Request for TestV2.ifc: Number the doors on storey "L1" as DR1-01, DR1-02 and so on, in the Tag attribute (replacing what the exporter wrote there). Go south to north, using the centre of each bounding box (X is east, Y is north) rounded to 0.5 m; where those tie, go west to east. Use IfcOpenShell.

First a look at what the model holds.

```python
import ifcopenshell
import ifcopenshell.util.element
import ifcopenshell.util.placement

model = ifcopenshell.open("TestV2.ifc")
print(model.schema)
storey = next(s for s in model.by_type("IfcBuildingStorey") if s.Name == "L1")
doors = [e for e in ifcopenshell.util.element.get_decomposition(storey) if e.is_a("IfcDoor")]
for e in sorted(doors, key=lambda e: e.id()):
    origin = ifcopenshell.util.placement.get_local_placement(e.ObjectPlacement)[:3, 3]
    print(e.id(), e.Tag, e.Name, origin.round(2) + 0.0, sep=" | ")
```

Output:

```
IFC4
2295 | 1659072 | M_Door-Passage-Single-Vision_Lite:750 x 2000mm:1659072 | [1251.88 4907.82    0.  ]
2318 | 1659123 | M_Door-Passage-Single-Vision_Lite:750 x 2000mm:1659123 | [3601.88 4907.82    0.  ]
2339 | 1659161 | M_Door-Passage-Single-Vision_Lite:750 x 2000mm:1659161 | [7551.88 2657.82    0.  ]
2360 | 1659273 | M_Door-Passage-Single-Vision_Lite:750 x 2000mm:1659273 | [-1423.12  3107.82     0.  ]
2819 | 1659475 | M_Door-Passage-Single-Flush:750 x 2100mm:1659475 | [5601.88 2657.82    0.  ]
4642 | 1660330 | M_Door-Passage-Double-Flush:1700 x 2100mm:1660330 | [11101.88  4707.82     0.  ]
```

```python
import ifcopenshell
import ifcopenshell.geom
import ifcopenshell.util.element
import ifcopenshell.util.shape

model = ifcopenshell.open("TestV2.ifc")
settings = ifcopenshell.geom.settings()
settings.set("use-world-coords", True)


def centre(element):
    shape = ifcopenshell.geom.create_shape(settings, element)
    return ifcopenshell.util.shape.get_bbox_centroid(shape.geometry)


storey = next(s for s in model.by_type("IfcBuildingStorey") if s.Name == "L1")
doors = [e for e in ifcopenshell.util.element.get_decomposition(storey) if e.is_a("IfcDoor")]

# Insertion points can sit at a corner or the storey origin, so sort by the geometry (in metres).
centres = {e: centre(e) for e in doors}
doors.sort(key=lambda e: (round(centres[e][1] / 0.5), centres[e][0]))

for i, e in enumerate(doors, start=1):
    number = f"DR1-{i:02d}"
    e.Tag = number
    print(e.id(), number)

model.write("TestV2_edited.ifc")
```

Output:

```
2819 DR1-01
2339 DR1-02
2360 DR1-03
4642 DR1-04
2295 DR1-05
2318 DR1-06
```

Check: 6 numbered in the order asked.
